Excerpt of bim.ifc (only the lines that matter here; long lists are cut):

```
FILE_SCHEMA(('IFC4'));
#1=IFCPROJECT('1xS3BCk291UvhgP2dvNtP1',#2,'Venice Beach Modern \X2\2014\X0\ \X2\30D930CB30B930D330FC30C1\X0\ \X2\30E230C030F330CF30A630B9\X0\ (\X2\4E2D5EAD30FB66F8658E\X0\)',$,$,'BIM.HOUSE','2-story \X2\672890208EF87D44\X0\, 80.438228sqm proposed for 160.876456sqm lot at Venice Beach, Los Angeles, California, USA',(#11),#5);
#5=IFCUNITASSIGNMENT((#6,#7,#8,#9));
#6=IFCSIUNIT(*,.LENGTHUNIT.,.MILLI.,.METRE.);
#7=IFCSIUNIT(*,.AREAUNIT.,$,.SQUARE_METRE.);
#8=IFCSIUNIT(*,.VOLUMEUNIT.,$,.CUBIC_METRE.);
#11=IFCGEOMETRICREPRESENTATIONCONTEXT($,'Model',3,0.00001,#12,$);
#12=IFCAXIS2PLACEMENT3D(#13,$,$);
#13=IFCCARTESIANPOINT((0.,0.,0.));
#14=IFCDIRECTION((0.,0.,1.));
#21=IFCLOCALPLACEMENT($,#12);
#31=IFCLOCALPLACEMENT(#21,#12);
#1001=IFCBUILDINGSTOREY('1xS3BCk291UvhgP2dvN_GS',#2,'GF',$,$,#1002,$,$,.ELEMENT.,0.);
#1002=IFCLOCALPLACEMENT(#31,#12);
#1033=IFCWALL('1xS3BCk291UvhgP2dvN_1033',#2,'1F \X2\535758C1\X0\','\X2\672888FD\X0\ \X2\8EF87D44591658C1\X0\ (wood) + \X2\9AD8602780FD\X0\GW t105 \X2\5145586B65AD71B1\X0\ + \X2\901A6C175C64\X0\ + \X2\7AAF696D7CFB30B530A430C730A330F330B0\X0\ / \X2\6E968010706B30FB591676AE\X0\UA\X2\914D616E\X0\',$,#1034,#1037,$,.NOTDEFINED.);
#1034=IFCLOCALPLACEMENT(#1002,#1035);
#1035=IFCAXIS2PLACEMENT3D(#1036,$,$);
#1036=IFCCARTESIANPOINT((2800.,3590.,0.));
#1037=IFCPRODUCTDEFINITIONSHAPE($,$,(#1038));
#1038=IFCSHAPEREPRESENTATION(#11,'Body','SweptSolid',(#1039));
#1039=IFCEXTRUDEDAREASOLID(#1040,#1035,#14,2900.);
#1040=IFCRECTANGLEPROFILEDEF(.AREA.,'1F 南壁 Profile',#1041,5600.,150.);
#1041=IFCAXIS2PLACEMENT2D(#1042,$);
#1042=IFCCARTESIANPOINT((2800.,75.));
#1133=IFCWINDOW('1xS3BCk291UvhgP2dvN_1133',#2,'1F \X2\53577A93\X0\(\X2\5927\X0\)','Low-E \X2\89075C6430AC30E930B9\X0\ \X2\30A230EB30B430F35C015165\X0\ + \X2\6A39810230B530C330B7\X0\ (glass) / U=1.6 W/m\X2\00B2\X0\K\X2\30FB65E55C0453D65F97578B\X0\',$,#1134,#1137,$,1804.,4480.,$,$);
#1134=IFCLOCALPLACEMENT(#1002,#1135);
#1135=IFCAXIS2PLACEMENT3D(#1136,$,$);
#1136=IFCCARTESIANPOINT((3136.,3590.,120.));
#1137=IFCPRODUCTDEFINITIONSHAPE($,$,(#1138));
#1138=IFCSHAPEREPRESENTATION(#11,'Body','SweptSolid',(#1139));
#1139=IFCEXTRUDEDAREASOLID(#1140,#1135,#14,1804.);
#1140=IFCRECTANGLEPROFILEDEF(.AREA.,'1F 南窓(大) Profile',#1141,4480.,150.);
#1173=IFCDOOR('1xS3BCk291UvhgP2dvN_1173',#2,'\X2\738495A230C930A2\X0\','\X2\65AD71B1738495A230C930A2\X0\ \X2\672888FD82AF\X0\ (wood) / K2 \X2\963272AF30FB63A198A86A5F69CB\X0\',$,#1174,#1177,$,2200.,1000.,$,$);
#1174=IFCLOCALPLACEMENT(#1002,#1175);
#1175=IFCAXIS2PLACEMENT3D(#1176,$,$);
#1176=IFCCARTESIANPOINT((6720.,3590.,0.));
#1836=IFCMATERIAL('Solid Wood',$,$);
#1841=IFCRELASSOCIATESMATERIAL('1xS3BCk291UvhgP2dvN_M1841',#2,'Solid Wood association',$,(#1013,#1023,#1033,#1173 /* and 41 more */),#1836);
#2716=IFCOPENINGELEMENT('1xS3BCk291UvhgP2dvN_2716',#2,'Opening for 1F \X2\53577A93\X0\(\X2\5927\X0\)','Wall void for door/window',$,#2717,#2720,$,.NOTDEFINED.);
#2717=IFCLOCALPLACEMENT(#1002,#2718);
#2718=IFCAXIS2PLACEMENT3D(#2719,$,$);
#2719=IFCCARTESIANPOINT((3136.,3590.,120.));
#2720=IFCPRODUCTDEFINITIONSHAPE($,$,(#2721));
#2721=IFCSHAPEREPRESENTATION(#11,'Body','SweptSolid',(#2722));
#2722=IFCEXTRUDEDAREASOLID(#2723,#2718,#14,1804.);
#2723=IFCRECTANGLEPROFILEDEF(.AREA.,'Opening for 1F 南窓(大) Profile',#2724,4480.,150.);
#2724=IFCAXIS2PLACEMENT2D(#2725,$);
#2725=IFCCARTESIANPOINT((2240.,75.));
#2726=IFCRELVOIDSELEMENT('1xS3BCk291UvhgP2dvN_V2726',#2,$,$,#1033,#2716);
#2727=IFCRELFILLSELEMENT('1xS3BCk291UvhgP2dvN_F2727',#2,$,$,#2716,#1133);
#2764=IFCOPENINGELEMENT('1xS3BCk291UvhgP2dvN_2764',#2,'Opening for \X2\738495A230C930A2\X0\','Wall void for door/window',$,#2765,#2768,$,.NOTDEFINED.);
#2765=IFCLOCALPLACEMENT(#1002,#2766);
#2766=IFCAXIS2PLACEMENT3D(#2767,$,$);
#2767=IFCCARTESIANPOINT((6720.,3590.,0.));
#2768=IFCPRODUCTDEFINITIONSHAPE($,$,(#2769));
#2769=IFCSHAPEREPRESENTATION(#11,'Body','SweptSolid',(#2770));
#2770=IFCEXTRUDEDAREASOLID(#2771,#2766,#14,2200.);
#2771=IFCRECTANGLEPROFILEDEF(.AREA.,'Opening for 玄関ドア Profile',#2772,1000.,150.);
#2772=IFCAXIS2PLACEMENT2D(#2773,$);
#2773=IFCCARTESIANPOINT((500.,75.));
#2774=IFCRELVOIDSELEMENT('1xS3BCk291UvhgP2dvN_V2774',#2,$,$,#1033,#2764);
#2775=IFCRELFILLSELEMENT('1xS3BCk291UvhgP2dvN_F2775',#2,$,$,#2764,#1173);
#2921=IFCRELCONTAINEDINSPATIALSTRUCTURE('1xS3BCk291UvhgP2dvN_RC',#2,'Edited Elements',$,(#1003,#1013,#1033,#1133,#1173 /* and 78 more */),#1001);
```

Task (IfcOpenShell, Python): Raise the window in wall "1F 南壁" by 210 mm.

```python
import numpy as np
import ifcopenshell
import ifcopenshell.api.geometry
import ifcopenshell.util.placement
import ifcopenshell.util.unit

model = ifcopenshell.open("bim.ifc")
unit_scale = ifcopenshell.util.unit.calculate_unit_scale(model)

window = model.by_guid("1xS3BCk291UvhgP2dvN_1133")
opening = window.FillsVoids[0].RelatingOpeningElement
dz = 210.0

shift = np.array([0.0, 0.0, dz])
# The window is not placed relative to its opening, so move both.
for product in (opening, window):
    matrix = ifcopenshell.util.placement.get_local_placement(product.ObjectPlacement)
    matrix[:3, 3] += shift
    ifcopenshell.api.geometry.edit_object_placement(model, product=product, matrix=matrix, is_si=False)

print(f"moved by {dz * unit_scale:+.3f} m")

model.write("bim_edited.ifc")
```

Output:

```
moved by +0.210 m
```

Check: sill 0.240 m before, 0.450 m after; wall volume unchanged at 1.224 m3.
